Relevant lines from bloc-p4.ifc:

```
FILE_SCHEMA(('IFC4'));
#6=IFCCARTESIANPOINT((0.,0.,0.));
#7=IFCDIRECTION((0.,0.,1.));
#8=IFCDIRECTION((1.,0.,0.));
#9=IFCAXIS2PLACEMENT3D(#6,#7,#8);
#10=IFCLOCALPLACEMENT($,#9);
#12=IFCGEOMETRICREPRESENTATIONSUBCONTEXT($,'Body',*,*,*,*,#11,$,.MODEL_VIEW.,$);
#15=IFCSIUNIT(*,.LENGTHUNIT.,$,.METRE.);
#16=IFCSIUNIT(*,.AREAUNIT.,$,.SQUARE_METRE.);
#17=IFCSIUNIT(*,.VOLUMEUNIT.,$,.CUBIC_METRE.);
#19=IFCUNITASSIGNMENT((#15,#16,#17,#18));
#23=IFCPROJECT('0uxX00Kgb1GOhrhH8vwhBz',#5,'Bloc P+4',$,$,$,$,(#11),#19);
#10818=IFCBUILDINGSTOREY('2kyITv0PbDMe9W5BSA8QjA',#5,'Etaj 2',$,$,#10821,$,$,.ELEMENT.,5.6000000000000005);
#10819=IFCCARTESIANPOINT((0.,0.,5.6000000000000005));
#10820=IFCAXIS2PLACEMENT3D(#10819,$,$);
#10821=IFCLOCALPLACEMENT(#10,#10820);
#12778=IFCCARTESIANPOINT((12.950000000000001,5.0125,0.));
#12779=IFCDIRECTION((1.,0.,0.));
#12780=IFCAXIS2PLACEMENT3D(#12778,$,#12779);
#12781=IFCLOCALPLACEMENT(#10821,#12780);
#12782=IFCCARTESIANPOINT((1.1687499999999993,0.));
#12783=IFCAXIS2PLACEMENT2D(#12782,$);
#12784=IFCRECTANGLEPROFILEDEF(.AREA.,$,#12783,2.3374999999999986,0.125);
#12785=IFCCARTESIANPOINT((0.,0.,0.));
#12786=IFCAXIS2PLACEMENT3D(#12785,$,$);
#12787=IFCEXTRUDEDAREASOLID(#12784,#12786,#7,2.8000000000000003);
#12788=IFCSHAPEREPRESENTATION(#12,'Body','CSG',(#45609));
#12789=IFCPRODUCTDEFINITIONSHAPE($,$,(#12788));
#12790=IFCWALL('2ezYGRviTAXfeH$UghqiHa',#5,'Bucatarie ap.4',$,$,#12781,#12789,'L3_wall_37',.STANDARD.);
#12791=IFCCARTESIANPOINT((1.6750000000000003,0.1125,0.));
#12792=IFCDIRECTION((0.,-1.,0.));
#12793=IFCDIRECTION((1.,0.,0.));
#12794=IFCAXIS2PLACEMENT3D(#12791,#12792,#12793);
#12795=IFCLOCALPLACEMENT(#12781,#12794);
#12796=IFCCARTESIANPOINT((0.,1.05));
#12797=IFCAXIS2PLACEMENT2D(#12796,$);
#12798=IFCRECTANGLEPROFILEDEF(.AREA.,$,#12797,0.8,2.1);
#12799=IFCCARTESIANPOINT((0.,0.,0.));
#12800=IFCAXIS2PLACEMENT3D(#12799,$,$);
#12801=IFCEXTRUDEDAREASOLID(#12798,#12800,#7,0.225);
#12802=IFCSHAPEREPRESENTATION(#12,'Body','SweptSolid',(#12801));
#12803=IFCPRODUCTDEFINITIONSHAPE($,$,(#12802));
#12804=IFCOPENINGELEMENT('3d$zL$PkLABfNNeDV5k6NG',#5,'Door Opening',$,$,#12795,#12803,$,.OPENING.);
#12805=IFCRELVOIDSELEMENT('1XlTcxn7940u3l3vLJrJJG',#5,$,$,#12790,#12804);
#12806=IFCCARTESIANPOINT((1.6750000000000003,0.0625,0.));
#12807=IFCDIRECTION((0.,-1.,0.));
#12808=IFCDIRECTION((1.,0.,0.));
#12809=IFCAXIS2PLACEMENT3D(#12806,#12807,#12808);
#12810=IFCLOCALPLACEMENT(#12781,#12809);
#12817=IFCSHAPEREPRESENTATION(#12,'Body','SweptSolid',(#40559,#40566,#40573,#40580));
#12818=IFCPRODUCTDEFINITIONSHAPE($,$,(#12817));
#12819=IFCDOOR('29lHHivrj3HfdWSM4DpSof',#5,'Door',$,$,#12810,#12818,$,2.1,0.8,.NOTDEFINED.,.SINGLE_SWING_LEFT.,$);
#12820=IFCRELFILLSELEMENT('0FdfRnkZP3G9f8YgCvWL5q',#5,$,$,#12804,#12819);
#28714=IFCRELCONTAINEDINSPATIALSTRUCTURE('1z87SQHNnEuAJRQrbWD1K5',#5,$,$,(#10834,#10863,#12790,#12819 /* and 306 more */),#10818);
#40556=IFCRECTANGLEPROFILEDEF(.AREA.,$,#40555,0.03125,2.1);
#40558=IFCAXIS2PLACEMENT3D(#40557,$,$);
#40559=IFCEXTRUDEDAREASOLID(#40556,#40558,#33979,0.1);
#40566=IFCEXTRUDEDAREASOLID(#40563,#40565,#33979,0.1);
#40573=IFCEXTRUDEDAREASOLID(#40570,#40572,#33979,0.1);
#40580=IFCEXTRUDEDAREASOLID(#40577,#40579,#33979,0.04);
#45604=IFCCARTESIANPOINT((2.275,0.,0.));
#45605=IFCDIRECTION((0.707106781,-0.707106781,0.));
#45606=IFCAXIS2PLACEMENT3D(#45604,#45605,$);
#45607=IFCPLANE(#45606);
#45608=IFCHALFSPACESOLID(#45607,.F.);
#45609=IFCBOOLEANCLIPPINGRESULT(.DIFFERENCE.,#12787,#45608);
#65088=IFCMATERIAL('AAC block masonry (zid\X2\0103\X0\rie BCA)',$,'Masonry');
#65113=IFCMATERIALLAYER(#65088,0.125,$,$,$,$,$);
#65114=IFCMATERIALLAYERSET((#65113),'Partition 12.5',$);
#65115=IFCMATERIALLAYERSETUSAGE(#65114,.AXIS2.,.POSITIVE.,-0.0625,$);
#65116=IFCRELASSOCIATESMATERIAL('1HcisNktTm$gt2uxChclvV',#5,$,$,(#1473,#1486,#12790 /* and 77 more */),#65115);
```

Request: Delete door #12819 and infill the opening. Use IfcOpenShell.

```python
import ifcopenshell
import ifcopenshell.api.feature
import ifcopenshell.api.root
import ifcopenshell.geom
import ifcopenshell.util.shape

model = ifcopenshell.open("bloc-p4.ifc")
settings = ifcopenshell.geom.settings()


def volume(element):
    """Net volume in cubic metres, openings subtracted."""
    shape = ifcopenshell.geom.create_shape(settings, element)
    return ifcopenshell.util.shape.get_volume(shape.geometry)


door = model.by_id(12819)
opening = door.FillsVoids[0].RelatingOpeningElement
wall = opening.VoidsElements[0].RelatingBuildingElement
before = volume(wall)

ifcopenshell.api.root.remove_product(model, product=door)
ifcopenshell.api.feature.remove_feature(model, feature=opening)

after = volume(wall)

print(f"wall volume {before:.3f} -> {after:.3f} m3")

model.write("bloc-p4_rev.ifc")
```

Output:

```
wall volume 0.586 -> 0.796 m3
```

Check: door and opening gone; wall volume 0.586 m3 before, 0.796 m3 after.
